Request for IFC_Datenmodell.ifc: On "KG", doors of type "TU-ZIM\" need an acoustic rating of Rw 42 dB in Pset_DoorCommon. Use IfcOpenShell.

First a look at what the model holds.

```python
import ifcopenshell
import ifcopenshell.util.element

model = ifcopenshell.open("IFC_Datenmodell.ifc")
print(model.schema)
storey = next(s for s in model.by_type("IfcBuildingStorey") if s.Name == "KG")
doors = [e for e in ifcopenshell.util.element.get_decomposition(storey) if e.is_a("IfcDoor")]
seen = {}
for e in doors:
    element_type = ifcopenshell.util.element.get_type(e)
    key = (element_type.Name if element_type != e and element_type else None, ifcopenshell.util.element.get_pset(e, "Pset_DoorCommon", "AcousticRating"))
    seen[key] = seen.get(key, 0) + 1
for (name, value), count in sorted(seen.items(), key=str):
    print(count, "x", name, "|", value)
```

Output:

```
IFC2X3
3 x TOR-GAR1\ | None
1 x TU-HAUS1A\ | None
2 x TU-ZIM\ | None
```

```python
import ifcopenshell
import ifcopenshell.api.pset
import ifcopenshell.util.element

model = ifcopenshell.open("IFC_Datenmodell.ifc")

storey = next(s for s in model.by_type("IfcBuildingStorey") if s.Name == "KG")
doors = [e for e in ifcopenshell.util.element.get_decomposition(storey) if e.is_a("IfcDoor")]

count = 0
for e in doors:
    element_type = ifcopenshell.util.element.get_type(e)
    if element_type in (None, e) or element_type.Name != 'TU-ZIM\\':
        continue
    # add_pset returns the element's existing set when there is one.
    pset = ifcopenshell.api.pset.add_pset(model, product=e, name="Pset_DoorCommon")
    ifcopenshell.api.pset.edit_pset(model, pset=pset, properties={"AcousticRating": "Rw 42 dB"})
    count += 1

print(count, "doors updated")

model.write("IFC_Datenmodell_rev.ifc")
```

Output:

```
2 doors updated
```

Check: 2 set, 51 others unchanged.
